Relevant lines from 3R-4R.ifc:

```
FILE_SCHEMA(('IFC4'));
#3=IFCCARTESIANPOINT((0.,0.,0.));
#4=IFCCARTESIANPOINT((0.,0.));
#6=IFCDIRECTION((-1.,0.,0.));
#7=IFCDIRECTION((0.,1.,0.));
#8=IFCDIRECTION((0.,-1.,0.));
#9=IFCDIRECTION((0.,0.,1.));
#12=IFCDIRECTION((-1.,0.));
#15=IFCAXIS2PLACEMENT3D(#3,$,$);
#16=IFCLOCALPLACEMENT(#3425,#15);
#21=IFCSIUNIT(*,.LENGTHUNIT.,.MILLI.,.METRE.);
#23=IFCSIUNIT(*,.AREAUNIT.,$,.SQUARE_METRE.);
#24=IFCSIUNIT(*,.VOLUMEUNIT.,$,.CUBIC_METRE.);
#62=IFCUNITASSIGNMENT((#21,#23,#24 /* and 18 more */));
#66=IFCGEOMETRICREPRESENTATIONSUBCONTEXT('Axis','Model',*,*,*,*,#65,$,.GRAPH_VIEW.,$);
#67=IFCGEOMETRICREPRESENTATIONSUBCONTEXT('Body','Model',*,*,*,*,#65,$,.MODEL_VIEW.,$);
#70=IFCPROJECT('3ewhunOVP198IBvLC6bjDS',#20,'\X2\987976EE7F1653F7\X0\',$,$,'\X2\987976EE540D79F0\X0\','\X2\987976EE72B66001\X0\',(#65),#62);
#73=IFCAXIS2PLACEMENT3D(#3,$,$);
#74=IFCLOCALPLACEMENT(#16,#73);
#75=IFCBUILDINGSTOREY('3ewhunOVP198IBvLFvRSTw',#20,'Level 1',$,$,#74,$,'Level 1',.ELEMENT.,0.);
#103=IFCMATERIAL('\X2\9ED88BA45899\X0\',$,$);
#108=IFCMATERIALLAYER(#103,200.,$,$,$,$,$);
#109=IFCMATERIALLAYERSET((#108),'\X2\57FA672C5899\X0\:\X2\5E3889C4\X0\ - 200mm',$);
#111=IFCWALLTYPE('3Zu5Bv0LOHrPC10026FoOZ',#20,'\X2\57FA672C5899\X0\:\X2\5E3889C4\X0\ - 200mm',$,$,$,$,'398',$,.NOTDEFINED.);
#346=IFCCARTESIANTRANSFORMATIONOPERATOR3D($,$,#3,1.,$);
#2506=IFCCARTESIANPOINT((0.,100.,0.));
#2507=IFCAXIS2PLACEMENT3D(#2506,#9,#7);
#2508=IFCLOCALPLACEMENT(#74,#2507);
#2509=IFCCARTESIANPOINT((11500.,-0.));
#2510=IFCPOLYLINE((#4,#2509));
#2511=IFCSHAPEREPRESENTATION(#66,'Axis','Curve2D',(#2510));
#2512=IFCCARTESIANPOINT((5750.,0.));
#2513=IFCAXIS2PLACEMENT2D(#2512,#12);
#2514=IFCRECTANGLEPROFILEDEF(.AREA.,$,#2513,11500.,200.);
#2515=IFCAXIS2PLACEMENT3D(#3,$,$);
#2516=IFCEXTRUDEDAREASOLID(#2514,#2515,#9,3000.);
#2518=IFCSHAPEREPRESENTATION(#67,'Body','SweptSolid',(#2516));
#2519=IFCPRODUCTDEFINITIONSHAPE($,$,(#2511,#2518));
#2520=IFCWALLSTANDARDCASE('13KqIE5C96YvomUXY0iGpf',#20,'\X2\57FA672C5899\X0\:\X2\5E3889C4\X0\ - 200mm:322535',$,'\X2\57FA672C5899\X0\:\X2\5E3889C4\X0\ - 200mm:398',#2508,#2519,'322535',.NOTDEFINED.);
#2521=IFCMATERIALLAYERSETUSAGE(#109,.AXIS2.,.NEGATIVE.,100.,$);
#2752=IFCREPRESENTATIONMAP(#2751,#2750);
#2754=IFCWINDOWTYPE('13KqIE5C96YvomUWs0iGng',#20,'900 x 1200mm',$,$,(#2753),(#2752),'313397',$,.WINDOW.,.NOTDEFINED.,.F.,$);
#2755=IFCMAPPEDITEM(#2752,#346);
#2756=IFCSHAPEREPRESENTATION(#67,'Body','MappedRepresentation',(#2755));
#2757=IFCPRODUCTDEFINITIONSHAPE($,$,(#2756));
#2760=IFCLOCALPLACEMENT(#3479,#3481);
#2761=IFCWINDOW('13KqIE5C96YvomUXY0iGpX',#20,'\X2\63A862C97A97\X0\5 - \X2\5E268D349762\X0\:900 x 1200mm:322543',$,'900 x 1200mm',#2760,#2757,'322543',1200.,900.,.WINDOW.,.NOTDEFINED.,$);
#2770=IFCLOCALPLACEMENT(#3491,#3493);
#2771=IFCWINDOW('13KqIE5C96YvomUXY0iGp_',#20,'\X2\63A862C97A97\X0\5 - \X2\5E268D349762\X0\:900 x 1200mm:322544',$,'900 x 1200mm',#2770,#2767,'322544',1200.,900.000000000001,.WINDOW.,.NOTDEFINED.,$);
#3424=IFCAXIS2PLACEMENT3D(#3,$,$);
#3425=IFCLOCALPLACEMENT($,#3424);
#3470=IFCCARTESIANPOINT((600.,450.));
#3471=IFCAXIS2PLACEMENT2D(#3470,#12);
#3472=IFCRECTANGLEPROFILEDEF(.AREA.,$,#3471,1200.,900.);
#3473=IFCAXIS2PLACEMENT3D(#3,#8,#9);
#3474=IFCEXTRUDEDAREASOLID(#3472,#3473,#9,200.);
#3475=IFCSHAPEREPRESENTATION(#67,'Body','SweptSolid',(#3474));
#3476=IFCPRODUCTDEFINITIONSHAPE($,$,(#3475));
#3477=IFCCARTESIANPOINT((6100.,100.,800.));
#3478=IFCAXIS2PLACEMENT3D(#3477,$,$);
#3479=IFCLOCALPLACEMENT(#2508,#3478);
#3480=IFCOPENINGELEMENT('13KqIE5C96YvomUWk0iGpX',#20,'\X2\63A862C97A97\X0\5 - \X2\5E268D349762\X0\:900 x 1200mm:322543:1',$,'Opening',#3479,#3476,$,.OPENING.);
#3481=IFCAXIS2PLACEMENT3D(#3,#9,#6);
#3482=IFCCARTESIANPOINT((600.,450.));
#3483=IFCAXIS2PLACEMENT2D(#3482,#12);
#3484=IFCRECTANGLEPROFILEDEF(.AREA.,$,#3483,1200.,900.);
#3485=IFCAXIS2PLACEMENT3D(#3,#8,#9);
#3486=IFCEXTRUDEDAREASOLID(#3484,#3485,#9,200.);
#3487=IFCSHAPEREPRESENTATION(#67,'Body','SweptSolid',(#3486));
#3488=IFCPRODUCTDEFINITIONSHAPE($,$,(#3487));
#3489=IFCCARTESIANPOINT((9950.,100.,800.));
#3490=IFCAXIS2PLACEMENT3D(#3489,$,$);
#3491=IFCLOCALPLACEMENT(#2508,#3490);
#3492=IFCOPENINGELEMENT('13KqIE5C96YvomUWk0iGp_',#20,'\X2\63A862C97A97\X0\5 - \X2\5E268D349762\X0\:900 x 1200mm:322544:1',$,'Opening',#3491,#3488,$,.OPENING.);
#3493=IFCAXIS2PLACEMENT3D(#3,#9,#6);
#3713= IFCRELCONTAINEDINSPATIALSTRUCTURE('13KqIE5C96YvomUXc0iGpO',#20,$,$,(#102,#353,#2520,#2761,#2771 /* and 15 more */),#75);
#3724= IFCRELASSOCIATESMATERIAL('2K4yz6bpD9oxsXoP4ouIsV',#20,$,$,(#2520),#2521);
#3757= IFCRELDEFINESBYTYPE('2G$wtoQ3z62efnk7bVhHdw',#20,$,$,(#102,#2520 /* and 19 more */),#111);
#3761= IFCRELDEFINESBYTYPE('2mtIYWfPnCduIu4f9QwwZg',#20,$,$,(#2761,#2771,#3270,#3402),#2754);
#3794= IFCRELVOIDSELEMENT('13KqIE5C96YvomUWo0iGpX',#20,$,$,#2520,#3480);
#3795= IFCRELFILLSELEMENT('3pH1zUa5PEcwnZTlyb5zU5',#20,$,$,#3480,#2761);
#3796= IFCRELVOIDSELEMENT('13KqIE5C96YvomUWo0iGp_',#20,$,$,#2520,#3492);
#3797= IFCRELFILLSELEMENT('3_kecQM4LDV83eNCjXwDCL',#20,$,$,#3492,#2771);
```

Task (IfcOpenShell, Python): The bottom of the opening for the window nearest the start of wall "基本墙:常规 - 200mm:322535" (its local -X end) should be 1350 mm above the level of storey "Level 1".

```python
import numpy as np
import ifcopenshell
import ifcopenshell.api.geometry
import ifcopenshell.geom
import ifcopenshell.util.element
import ifcopenshell.util.placement
import ifcopenshell.util.shape
import ifcopenshell.util.unit

model = ifcopenshell.open("3R-4R.ifc")
unit_scale = ifcopenshell.util.unit.calculate_unit_scale(model)

window = model.by_guid("13KqIE5C96YvomUXY0iGpX")
opening = window.FillsVoids[0].RelatingOpeningElement
storey = ifcopenshell.util.element.get_container(window, ifc_class="IfcBuildingStorey")
level = ifcopenshell.util.placement.get_local_placement(storey.ObjectPlacement)[2, 3]

# The opening's origin need not be at the sill, so measure its lowest point.
shape = ifcopenshell.geom.create_shape(ifcopenshell.geom.settings(), opening)
bottom = ifcopenshell.util.shape.get_shape_bottom_elevation(shape, shape.geometry) / unit_scale
dz = level + 1.35 / unit_scale - bottom

shift = np.array([0.0, 0.0, dz])
# The window is placed relative to its opening, so it follows when the opening moves.
matrix = ifcopenshell.util.placement.get_local_placement(opening.ObjectPlacement)
matrix[:3, 3] += shift
ifcopenshell.api.geometry.edit_object_placement(
    model, product=opening, matrix=matrix, is_si=False, should_transform_children=True
)

print(f"moved by {dz * unit_scale:+.3f} m")

model.write("3R-4R_updated.ifc")
```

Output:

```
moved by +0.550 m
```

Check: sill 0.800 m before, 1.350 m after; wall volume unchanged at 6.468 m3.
